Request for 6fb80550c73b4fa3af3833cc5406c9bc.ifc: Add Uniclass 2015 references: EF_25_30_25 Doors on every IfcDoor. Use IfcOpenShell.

First a look at what the model holds.

```python
import ifcopenshell

model = ifcopenshell.open("6fb80550c73b4fa3af3833cc5406c9bc.ifc")
print(model.schema)
print("classifications:", [c.Name for c in model.by_type("IfcClassification")])
for ifc_class in ("IfcDoor", "IfcRoof", "IfcStair", "IfcWall", "IfcWindow"):
    print(ifc_class, len(model.by_type(ifc_class)))
```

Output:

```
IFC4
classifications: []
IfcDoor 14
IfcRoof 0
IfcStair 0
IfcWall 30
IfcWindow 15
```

```python
import ifcopenshell
import ifcopenshell.api.classification

model = ifcopenshell.open("6fb80550c73b4fa3af3833cc5406c9bc.ifc")

system = ifcopenshell.api.classification.add_classification(model, classification="Uniclass 2015")

codes = {
    "IfcDoor": ("EF_25_30_25", "Doors"),
}
for ifc_class, (code, name) in codes.items():
    products = model.by_type(ifc_class)
    ifcopenshell.api.classification.add_reference(
        model, products=products, classification=system, identification=code, name=name
    )
    print(code, len(products))

model.write("6fb80550c73b4fa3af3833cc5406c9bc_v2.ifc")
```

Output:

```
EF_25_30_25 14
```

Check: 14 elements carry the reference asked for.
